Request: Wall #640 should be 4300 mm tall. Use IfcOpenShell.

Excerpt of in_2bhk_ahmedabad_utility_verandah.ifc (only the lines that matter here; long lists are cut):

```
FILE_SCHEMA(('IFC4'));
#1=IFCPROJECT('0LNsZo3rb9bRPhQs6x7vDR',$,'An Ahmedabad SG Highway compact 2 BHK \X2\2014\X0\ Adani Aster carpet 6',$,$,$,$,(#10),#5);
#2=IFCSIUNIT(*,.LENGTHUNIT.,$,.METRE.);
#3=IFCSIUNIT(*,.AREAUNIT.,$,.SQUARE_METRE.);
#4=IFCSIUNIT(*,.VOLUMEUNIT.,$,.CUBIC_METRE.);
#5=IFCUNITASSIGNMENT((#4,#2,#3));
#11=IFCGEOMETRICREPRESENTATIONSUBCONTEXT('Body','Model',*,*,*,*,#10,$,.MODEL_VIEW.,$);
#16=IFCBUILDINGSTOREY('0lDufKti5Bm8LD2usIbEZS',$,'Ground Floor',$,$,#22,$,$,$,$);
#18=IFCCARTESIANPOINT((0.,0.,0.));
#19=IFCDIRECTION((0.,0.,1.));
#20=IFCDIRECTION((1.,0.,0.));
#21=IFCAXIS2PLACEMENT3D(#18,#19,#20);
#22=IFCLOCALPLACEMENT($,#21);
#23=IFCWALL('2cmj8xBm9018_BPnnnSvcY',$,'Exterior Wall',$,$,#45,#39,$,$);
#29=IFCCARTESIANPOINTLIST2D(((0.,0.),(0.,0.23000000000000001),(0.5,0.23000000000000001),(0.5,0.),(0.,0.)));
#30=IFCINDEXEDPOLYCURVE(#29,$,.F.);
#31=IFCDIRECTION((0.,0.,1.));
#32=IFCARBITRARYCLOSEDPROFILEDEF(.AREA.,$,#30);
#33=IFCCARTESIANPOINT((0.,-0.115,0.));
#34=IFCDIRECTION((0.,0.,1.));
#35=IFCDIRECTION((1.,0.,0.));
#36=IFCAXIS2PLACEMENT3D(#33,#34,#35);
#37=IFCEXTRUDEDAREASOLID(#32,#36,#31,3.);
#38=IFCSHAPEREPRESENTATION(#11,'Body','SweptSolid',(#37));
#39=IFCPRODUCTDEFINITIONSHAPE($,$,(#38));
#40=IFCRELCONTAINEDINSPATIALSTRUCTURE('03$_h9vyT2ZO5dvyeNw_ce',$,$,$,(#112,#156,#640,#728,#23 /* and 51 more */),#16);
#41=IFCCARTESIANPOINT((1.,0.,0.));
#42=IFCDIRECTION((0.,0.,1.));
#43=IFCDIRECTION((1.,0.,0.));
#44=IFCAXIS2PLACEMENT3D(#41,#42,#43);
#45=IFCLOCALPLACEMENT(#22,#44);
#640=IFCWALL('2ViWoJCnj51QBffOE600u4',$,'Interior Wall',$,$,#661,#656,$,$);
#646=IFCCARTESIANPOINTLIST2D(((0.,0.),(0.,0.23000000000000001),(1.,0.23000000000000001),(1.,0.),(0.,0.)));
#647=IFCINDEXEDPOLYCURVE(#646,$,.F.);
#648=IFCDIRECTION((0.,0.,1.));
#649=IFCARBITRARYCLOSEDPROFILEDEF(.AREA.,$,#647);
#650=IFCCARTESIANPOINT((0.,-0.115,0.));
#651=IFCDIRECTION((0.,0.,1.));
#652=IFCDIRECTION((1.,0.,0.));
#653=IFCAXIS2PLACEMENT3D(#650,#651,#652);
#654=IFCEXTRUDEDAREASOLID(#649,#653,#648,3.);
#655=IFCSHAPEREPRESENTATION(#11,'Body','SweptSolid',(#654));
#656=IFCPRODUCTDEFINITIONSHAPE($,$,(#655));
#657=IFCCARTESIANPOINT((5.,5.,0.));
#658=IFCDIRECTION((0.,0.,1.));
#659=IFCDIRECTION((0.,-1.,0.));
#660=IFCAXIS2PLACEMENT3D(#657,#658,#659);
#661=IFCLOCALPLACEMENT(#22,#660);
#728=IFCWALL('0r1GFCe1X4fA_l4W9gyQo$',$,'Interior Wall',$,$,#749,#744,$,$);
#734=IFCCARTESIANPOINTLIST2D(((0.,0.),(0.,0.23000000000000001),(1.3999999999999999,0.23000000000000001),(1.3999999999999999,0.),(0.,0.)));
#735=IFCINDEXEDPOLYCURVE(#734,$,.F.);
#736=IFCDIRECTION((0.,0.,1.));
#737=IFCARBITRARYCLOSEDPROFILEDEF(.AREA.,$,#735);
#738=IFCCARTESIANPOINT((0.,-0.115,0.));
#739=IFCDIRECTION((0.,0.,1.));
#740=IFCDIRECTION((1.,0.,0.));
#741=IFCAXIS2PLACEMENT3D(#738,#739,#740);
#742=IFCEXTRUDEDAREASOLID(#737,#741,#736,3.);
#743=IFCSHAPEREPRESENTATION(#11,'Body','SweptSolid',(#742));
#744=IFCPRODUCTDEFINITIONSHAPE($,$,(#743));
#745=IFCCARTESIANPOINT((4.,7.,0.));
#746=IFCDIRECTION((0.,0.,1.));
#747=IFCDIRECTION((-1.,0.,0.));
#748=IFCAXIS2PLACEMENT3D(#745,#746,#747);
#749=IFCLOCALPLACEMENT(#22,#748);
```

```python
import ifcopenshell
import ifcopenshell.geom
import ifcopenshell.util.representation
import ifcopenshell.util.shape

model = ifcopenshell.open("in_2bhk_ahmedabad_utility_verandah.ifc")
settings = ifcopenshell.geom.settings()


def volume(element):
    """Net volume in cubic metres, openings subtracted."""
    shape = ifcopenshell.geom.create_shape(settings, element)
    return ifcopenshell.util.shape.get_volume(shape.geometry)


wall = model.by_guid("2ViWoJCnj51QBffOE600u4")
before = volume(wall)

body = ifcopenshell.util.representation.get_representation(wall, "Model", "Body")
solid = body.Items[0]
old_height = solid.Depth
solid.Depth = 4.3
after = volume(wall)

print(f"height {old_height:g} -> {solid.Depth:g}, volume {before:.3f} -> {after:.3f} m3")

model.write("in_2bhk_ahmedabad_utility_verandah_rev.ifc")
```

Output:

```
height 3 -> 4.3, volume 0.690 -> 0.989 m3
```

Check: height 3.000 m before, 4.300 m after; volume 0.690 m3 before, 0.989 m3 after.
